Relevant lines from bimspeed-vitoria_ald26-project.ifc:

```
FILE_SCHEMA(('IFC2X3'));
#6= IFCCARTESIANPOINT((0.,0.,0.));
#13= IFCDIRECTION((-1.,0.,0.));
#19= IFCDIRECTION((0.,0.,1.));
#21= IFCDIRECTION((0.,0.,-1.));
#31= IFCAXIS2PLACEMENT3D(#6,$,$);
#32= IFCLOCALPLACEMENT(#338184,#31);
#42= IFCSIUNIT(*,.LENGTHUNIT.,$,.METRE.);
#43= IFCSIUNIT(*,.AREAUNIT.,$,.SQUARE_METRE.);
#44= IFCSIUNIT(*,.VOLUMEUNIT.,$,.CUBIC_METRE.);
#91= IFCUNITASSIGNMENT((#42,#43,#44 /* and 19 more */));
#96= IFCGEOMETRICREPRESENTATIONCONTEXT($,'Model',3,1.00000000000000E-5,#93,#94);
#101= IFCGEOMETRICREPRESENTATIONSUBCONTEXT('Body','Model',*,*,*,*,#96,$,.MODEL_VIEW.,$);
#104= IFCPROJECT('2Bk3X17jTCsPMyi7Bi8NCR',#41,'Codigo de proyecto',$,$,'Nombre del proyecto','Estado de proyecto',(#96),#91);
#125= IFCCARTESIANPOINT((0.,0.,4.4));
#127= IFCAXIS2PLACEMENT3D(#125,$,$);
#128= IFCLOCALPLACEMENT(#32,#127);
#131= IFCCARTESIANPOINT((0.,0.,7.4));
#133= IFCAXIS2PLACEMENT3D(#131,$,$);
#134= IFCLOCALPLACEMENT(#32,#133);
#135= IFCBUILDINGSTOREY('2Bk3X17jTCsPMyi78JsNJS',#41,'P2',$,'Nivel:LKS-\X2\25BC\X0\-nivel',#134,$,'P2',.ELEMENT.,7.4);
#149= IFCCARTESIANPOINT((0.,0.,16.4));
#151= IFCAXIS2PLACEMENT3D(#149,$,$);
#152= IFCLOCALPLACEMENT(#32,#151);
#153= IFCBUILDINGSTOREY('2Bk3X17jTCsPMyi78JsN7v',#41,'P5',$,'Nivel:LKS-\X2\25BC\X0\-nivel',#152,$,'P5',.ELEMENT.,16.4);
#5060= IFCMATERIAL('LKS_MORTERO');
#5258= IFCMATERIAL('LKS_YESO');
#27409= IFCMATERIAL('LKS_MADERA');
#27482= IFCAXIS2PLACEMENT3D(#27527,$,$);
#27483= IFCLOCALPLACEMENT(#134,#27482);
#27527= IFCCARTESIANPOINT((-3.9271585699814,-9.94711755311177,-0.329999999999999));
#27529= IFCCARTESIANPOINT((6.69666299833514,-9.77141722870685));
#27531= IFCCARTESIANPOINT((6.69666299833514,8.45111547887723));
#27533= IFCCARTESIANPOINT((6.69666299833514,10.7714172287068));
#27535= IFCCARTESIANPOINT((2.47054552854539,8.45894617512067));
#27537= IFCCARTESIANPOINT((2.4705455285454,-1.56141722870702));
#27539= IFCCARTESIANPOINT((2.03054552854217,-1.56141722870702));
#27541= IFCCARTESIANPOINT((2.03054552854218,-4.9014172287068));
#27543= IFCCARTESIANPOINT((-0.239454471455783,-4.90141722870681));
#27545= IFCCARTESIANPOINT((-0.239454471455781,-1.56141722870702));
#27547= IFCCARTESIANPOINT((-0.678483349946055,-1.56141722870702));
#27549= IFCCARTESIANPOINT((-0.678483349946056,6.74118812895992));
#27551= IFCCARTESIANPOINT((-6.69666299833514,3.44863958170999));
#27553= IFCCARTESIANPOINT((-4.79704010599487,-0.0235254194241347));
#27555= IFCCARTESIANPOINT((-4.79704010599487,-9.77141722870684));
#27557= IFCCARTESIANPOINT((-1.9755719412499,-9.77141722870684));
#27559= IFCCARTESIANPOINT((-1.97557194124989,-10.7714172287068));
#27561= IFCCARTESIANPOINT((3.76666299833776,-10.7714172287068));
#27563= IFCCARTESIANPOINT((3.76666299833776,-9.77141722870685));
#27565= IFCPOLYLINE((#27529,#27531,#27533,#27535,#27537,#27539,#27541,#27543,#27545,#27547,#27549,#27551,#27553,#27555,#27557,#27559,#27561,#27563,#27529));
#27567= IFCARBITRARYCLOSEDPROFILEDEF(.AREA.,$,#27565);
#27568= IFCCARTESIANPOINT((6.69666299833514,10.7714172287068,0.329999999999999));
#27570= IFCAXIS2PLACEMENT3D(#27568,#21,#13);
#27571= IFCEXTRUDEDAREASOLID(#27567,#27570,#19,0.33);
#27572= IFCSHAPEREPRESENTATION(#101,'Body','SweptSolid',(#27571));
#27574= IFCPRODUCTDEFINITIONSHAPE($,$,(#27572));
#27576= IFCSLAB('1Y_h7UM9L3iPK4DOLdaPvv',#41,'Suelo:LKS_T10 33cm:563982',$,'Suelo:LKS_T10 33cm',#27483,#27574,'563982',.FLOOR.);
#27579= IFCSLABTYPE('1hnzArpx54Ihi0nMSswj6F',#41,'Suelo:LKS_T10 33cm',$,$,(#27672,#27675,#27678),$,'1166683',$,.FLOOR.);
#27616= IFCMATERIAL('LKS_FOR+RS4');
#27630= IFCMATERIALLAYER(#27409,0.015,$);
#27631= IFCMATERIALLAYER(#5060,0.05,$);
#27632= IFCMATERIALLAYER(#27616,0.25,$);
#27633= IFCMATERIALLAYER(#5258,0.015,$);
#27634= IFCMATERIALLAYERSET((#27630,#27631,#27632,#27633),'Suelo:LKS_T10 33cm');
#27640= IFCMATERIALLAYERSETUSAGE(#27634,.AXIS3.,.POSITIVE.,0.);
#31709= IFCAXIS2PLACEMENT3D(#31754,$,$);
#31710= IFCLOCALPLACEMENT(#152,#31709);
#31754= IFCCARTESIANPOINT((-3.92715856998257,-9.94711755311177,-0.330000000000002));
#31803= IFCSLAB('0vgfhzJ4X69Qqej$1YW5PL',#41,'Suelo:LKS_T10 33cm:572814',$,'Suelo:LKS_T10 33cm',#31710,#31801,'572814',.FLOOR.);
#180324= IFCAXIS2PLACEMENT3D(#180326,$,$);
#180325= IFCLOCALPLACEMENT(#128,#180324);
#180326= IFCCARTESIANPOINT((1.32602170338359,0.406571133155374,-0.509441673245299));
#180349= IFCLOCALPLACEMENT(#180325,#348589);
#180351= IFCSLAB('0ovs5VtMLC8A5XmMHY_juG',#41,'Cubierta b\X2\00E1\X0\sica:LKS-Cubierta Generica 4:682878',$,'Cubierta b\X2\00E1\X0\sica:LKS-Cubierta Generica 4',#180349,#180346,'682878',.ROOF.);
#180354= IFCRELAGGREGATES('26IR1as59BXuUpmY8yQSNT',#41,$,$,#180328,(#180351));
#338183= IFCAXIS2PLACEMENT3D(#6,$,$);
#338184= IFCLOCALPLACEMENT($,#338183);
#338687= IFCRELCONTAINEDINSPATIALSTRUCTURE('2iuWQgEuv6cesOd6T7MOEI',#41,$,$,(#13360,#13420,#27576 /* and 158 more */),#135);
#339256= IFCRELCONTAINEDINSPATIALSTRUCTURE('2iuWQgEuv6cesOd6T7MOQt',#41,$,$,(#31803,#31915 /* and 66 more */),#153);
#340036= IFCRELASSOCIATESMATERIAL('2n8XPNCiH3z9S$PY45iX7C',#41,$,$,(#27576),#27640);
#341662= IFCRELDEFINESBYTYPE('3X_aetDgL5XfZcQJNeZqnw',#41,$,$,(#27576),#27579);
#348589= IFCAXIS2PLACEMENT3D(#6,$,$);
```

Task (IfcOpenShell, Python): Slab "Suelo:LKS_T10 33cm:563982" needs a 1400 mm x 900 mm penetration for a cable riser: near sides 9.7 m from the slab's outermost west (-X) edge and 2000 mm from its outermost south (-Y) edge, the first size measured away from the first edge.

```python
import numpy as np
import ifcopenshell
import ifcopenshell.api.feature
import ifcopenshell.api.geometry
import ifcopenshell.api.root
import ifcopenshell.geom
import ifcopenshell.util.placement
import ifcopenshell.util.representation
import ifcopenshell.util.shape
import ifcopenshell.util.unit

model = ifcopenshell.open("bimspeed-vitoria_ald26-project.ifc")
unit_scale = ifcopenshell.util.unit.calculate_unit_scale(model)
settings = ifcopenshell.geom.settings()


def volume(element):
    """Net volume in cubic metres, openings subtracted."""
    shape = ifcopenshell.geom.create_shape(settings, element)
    return ifcopenshell.util.shape.get_volume(shape.geometry)


slab = model.by_guid("1Y_h7UM9L3iPK4DOLdaPvv")
before = volume(slab)

# Extent in the slab's own axes, in metres. The edges named are its -X and -Y sides.
slab_shape = ifcopenshell.geom.create_shape(settings, slab)
vertices = ifcopenshell.util.shape.get_vertices(slab_shape.geometry)
x_min, y_min, bottom = vertices.min(axis=0)
top = vertices[:, 2].max()

opening = ifcopenshell.api.root.create_entity(model, ifc_class="IfcOpeningElement", name="Cable riser opening")
context = ifcopenshell.util.representation.get_context(model, "Model", "Body", "MODEL_VIEW")
width, depth = 1.4, 0.9
outline = [(0.0, 0.0), (width, 0.0), (width, depth), (0.0, depth), (0.0, 0.0)]
# Overshoot both faces by 50 mm so the cut is clean.
shape = ifcopenshell.api.geometry.add_slab_representation(
    model, context=context, depth=top - bottom + 0.1, polyline=outline
)
ifcopenshell.api.geometry.assign_representation(model, product=opening, representation=shape)

matrix = ifcopenshell.util.placement.get_local_placement(slab.ObjectPlacement)
matrix[:, 3] = matrix @ np.append(np.array([x_min + 9.7, y_min + 2, bottom - 0.05]) / unit_scale, 1.0)
ifcopenshell.api.geometry.edit_object_placement(model, product=opening, matrix=matrix, is_si=False)
ifcopenshell.api.feature.add_feature(model, feature=opening, element=slab)

after = volume(slab)

print(f"slab volume {before:.3f} -> {after:.3f} m3")

model.write("bimspeed-vitoria_ald26-project_edited.ifc")
```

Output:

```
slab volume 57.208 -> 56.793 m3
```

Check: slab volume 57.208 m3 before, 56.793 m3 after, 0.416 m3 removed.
